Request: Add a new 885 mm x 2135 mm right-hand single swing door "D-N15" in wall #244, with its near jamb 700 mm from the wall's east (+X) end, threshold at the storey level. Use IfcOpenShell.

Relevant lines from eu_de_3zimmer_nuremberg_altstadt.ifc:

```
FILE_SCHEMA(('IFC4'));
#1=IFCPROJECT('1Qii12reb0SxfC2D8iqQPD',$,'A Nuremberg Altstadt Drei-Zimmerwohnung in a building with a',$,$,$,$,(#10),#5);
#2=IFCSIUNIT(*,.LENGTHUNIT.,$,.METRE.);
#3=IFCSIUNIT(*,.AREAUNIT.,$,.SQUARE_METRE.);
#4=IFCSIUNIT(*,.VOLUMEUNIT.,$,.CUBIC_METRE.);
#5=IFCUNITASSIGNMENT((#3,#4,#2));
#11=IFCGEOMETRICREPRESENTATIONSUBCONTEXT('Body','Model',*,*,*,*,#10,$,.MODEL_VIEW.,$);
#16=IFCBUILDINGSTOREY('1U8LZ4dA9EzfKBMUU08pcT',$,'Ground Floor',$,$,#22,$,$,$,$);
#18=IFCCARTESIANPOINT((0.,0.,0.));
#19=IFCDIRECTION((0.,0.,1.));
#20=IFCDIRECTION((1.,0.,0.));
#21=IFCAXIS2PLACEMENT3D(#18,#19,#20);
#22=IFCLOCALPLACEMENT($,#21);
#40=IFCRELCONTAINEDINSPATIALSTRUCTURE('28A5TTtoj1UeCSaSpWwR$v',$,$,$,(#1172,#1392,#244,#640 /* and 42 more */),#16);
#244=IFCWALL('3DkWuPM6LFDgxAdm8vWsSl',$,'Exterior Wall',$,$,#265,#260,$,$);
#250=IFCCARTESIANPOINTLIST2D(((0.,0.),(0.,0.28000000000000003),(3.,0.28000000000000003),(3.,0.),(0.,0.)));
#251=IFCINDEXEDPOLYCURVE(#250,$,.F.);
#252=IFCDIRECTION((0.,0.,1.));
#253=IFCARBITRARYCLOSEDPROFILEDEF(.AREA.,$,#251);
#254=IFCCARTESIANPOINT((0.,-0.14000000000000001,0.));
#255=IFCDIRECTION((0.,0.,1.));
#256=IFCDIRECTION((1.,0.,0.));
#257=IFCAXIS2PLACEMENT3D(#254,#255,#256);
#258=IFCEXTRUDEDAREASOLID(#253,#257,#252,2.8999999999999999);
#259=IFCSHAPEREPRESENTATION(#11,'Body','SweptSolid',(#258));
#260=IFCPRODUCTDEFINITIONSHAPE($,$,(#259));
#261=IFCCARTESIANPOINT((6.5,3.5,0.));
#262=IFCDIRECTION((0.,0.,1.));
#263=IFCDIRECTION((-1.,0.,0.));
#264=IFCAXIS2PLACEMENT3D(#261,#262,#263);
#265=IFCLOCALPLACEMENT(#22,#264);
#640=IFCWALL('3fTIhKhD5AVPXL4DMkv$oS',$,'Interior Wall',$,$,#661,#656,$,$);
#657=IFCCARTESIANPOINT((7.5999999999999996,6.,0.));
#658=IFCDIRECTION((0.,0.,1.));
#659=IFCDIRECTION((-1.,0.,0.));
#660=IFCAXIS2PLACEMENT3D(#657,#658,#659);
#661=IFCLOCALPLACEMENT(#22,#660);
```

```python
import numpy as np
import ifcopenshell
import ifcopenshell.api.feature
import ifcopenshell.api.geometry
import ifcopenshell.api.root
import ifcopenshell.api.spatial
import ifcopenshell.geom
import ifcopenshell.util.element
import ifcopenshell.util.placement
import ifcopenshell.util.representation
import ifcopenshell.util.shape
import ifcopenshell.util.unit

model = ifcopenshell.open("eu_de_3zimmer_nuremberg_altstadt.ifc")
unit_scale = ifcopenshell.util.unit.calculate_unit_scale(model)
settings = ifcopenshell.geom.settings()


def volume(element):
    """Net volume in cubic metres, openings subtracted."""
    shape = ifcopenshell.geom.create_shape(settings, element)
    return ifcopenshell.util.shape.get_volume(shape.geometry)


wall = model.by_guid("3DkWuPM6LFDgxAdm8vWsSl")
storey = ifcopenshell.util.element.get_container(wall, ifc_class="IfcBuildingStorey")
context = ifcopenshell.util.representation.get_context(model, "Model", "Body", "MODEL_VIEW")
before = volume(wall)

width, height, from_end, sill = 0.885, 2.135, 0.7, 0.0  # metres

# The wall runs along its own X axis, and the end named is its -X end.
wall_shape = ifcopenshell.geom.create_shape(settings, wall)
x, y, z = ifcopenshell.util.shape.get_vertices(wall_shape.geometry).T
start = x.min() + from_end
face, thickness = float(y.min()), float(y.max() - y.min())
wall_matrix = ifcopenshell.util.placement.get_local_placement(wall.ObjectPlacement)
level = ifcopenshell.util.placement.get_local_placement(storey.ObjectPlacement)[2, 3]


def in_wall(x, y):
    """Placement at x, y metres in the wall's axes, at sill height."""
    matrix = wall_matrix.copy()
    matrix[:, 3] = wall_matrix @ np.array([x / unit_scale, y / unit_scale, 0.0, 1.0])
    matrix[2, 3] = level + sill / unit_scale
    return matrix


# Opening: a box that overshoots both wall faces by 50 mm.
opening = ifcopenshell.api.root.create_entity(model, ifc_class="IfcOpeningElement", predefined_type="OPENING")
box = ifcopenshell.api.geometry.add_wall_representation(
    model, context=context, length=width, height=height, thickness=thickness + 0.1
)
ifcopenshell.api.geometry.assign_representation(model, product=opening, representation=box)
ifcopenshell.api.geometry.edit_object_placement(model, product=opening, matrix=in_wall(start, face - 0.05), is_si=False)
ifcopenshell.api.feature.add_feature(model, feature=opening, element=wall)

door = ifcopenshell.api.root.create_entity(model, ifc_class="IfcDoor", name="D-N15", predefined_type="DOOR")
door.OverallWidth, door.OverallHeight = width / unit_scale, height / unit_scale
door.OperationType = "SINGLE_SWING_RIGHT"
body = ifcopenshell.api.geometry.add_door_representation(
    model,
    context=context,
    overall_width=door.OverallWidth,
    overall_height=door.OverallHeight,
    operation_type="SINGLE_SWING_RIGHT",
    lining_properties={"LiningDepth": thickness / unit_scale, "ThresholdDepth": thickness / unit_scale},
)
ifcopenshell.api.geometry.assign_representation(model, product=door, representation=body)
ifcopenshell.api.spatial.assign_container(model, products=[door], relating_structure=storey)
ifcopenshell.api.feature.add_filling(model, opening=opening, element=door)

# The lining spans the wall, so the door starts at the wall face.
ifcopenshell.api.geometry.edit_object_placement(model, product=door, matrix=in_wall(start, face), is_si=False)

after = volume(wall)

print(f"wall volume {before:.3f} -> {after:.3f} m3")

model.write("eu_de_3zimmer_nuremberg_altstadt-out.ifc")
```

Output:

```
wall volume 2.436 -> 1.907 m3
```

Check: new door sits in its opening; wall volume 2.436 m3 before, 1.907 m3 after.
